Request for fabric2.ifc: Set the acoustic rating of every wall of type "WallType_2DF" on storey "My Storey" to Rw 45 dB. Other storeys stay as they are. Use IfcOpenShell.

First a look at what the model holds.

```python
import ifcopenshell
import ifcopenshell.util.element

model = ifcopenshell.open("fabric2.ifc")
print(model.schema)
storey = next(s for s in model.by_type("IfcBuildingStorey") if s.Name == "My Storey")
walls = [e for e in ifcopenshell.util.element.get_decomposition(storey) if e.is_a("IfcWall")]
seen = {}
for e in walls:
    element_type = ifcopenshell.util.element.get_type(e)
    key = (element_type.Name if element_type != e and element_type else None, ifcopenshell.util.element.get_pset(e, "Pset_WallCommon", "AcousticRating"))
    seen[key] = seen.get(key, 0) + 1
for (name, value), count in sorted(seen.items(), key=str):
    print(count, "x", name, "|", value)
```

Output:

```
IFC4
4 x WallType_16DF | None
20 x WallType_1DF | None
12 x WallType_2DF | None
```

```python
import ifcopenshell
import ifcopenshell.api.pset
import ifcopenshell.util.element

model = ifcopenshell.open("fabric2.ifc")

storey = next(s for s in model.by_type("IfcBuildingStorey") if s.Name == "My Storey")
walls = [e for e in ifcopenshell.util.element.get_decomposition(storey) if e.is_a("IfcWall")]

count = 0
for e in walls:
    element_type = ifcopenshell.util.element.get_type(e)
    if element_type in (None, e) or element_type.Name != "WallType_2DF":
        continue
    # add_pset returns the element's existing set when there is one.
    pset = ifcopenshell.api.pset.add_pset(model, product=e, name="Pset_WallCommon")
    ifcopenshell.api.pset.edit_pset(model, pset=pset, properties={"AcousticRating": "Rw 45 dB"})
    count += 1

print(count, "walls updated")

model.write("fabric2_edited.ifc")
```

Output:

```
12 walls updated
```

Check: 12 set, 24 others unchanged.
